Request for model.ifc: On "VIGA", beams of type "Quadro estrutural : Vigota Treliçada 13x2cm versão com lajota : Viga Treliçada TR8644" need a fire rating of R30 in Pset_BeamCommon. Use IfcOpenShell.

First a look at what the model holds.

```python
import ifcopenshell
import ifcopenshell.util.element

model = ifcopenshell.open("model.ifc")
print(model.schema)
storey = next(s for s in model.by_type("IfcBuildingStorey") if s.Name == "VIGA")
beams = [e for e in ifcopenshell.util.element.get_decomposition(storey) if e.is_a("IfcBeam")]
seen = {}
for e in beams:
    element_type = ifcopenshell.util.element.get_type(e)
    key = (element_type.Name if element_type != e and element_type else None, ifcopenshell.util.element.get_pset(e, "Pset_BeamCommon", "FireRating"))
    seen[key] = seen.get(key, 0) + 1
for (name, value), count in sorted(seen.items(), key=str):
    print(count, "x", name, "|", value)
```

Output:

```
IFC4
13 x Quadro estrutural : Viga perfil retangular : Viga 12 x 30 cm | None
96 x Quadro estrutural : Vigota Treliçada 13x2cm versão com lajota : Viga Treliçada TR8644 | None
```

```python
import ifcopenshell
import ifcopenshell.api.pset
import ifcopenshell.util.element

model = ifcopenshell.open("model.ifc")

storey = next(s for s in model.by_type("IfcBuildingStorey") if s.Name == "VIGA")
beams = [e for e in ifcopenshell.util.element.get_decomposition(storey) if e.is_a("IfcBeam")]

count = 0
for e in beams:
    element_type = ifcopenshell.util.element.get_type(e)
    if element_type in (None, e) or element_type.Name != "Quadro estrutural : Vigota Treliçada 13x2cm versão com lajota : Viga Treliçada TR8644":
        continue
    # add_pset returns the element's existing set when there is one.
    pset = ifcopenshell.api.pset.add_pset(model, product=e, name="Pset_BeamCommon")
    ifcopenshell.api.pset.edit_pset(model, pset=pset, properties={"FireRating": "R30"})
    count += 1

print(count, "beams updated")

model.write("model_rev.ifc")
```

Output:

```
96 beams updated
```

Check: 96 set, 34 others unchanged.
